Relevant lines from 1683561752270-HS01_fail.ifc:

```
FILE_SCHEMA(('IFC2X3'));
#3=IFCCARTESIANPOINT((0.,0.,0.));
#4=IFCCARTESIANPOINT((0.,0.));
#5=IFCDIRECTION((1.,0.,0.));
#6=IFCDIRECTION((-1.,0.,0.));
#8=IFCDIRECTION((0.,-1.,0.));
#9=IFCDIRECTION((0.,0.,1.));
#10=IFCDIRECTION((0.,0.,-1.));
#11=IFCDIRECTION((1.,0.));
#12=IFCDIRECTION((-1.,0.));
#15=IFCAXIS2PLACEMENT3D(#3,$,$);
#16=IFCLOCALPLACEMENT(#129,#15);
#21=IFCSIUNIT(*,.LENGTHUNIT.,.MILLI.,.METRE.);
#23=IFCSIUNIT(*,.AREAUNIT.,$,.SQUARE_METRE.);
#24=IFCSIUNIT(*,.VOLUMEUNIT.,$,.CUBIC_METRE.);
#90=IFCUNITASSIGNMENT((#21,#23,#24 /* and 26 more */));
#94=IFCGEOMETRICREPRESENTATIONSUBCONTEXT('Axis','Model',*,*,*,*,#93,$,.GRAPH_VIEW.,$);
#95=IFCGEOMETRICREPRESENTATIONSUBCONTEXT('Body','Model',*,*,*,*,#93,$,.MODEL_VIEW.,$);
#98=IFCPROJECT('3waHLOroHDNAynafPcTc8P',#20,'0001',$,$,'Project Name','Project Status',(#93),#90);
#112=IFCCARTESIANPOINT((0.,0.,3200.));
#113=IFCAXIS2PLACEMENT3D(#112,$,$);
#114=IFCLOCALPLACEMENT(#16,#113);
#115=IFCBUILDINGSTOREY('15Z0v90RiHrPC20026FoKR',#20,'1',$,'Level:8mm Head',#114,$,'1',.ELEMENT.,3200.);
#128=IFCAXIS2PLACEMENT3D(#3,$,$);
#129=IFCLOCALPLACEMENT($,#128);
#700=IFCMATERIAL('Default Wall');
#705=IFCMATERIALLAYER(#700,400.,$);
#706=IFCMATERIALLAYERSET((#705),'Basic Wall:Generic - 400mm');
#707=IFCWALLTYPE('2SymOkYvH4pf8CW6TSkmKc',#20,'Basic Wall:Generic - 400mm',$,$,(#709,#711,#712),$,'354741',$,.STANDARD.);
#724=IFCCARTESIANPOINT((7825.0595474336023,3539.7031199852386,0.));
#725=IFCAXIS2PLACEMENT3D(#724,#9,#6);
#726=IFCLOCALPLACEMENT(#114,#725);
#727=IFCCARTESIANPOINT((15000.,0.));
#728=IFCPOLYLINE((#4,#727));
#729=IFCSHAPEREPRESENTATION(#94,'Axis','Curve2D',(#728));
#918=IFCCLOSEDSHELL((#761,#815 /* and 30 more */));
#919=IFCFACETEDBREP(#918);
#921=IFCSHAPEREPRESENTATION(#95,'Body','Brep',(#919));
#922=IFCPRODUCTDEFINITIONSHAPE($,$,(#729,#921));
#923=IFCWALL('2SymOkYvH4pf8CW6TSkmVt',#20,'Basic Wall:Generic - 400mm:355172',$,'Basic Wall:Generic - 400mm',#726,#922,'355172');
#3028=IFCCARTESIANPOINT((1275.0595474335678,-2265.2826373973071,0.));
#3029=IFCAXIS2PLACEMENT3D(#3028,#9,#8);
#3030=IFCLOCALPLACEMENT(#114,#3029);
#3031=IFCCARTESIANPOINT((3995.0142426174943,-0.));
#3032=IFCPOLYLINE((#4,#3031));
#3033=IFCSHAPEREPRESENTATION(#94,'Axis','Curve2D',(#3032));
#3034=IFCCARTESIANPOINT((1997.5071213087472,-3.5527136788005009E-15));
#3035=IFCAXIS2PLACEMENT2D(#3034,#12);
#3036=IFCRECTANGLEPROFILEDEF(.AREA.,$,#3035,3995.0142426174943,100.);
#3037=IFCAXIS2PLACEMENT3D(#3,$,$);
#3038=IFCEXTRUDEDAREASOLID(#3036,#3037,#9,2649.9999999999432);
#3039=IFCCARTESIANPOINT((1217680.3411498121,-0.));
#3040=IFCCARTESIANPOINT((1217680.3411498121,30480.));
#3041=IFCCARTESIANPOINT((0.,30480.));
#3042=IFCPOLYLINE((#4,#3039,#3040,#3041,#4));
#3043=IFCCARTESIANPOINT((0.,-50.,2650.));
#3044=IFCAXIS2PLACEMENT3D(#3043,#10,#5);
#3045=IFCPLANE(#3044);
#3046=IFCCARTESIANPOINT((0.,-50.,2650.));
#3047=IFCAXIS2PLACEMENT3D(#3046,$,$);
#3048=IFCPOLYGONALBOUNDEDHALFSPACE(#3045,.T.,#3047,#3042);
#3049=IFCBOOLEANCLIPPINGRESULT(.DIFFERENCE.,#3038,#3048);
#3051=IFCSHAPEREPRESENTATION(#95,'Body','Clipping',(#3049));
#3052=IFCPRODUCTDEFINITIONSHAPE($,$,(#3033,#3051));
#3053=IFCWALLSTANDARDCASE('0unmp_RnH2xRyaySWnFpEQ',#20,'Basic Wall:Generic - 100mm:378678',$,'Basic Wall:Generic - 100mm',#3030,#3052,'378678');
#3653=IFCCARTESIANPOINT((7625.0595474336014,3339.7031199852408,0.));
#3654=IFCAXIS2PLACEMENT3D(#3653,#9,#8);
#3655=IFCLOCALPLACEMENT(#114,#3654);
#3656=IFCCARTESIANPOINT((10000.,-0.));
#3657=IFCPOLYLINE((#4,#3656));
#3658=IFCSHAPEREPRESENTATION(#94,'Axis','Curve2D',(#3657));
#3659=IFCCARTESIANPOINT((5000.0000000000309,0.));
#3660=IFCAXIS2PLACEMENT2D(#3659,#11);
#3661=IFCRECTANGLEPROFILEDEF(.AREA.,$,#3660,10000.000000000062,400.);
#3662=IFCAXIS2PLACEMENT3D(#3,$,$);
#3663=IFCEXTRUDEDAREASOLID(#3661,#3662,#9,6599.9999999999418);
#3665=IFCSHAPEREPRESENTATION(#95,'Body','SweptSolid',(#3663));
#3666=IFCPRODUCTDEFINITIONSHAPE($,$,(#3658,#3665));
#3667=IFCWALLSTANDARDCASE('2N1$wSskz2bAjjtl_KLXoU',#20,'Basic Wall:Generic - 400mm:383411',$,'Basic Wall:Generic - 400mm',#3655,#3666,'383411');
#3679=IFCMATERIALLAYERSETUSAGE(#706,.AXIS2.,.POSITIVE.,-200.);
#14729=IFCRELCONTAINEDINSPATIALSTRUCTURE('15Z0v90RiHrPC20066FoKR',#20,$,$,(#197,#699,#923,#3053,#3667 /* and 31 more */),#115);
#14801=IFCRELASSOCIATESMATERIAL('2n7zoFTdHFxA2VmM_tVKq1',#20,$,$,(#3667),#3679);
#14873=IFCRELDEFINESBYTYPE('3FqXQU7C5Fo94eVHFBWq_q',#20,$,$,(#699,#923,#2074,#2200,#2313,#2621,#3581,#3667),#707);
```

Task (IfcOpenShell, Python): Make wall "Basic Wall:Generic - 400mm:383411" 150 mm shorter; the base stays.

```python
import ifcopenshell
import ifcopenshell.geom
import ifcopenshell.util.representation
import ifcopenshell.util.shape

model = ifcopenshell.open("1683561752270-HS01_fail.ifc")
settings = ifcopenshell.geom.settings()


def volume(element):
    """Net volume in cubic metres, openings subtracted."""
    shape = ifcopenshell.geom.create_shape(settings, element)
    return ifcopenshell.util.shape.get_volume(shape.geometry)


wall = model.by_id(3667)
before = volume(wall)

body = ifcopenshell.util.representation.get_representation(wall, "Model", "Body")
solid = body.Items[0]
old_height = solid.Depth
solid.Depth -= 150.0
after = volume(wall)

print(f"height {old_height:g} -> {solid.Depth:g}, volume {before:.3f} -> {after:.3f} m3")

model.write("1683561752270-HS01_fail-out.ifc")
```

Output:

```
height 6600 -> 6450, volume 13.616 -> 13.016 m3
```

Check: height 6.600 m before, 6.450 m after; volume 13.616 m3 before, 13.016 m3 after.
